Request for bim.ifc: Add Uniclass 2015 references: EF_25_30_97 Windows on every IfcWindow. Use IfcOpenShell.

First a look at what the model holds.

```python
import ifcopenshell

model = ifcopenshell.open("bim.ifc")
print(model.schema)
print("classifications:", [c.Name for c in model.by_type("IfcClassification")])
for ifc_class in ("IfcDoor", "IfcRoof", "IfcStair", "IfcWall", "IfcWindow"):
    print(ifc_class, len(model.by_type(ifc_class)))
```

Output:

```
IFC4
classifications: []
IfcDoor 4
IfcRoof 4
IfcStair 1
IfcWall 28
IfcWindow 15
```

```python
import ifcopenshell
import ifcopenshell.api.classification

model = ifcopenshell.open("bim.ifc")

system = ifcopenshell.api.classification.add_classification(model, classification="Uniclass 2015")

codes = {
    "IfcWindow": ("EF_25_30_97", "Windows"),
}
for ifc_class, (code, name) in codes.items():
    products = model.by_type(ifc_class)
    ifcopenshell.api.classification.add_reference(
        model, products=products, classification=system, identification=code, name=name
    )
    print(code, len(products))

model.write("bim_updated.ifc")
```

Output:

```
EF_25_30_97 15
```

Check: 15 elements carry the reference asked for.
